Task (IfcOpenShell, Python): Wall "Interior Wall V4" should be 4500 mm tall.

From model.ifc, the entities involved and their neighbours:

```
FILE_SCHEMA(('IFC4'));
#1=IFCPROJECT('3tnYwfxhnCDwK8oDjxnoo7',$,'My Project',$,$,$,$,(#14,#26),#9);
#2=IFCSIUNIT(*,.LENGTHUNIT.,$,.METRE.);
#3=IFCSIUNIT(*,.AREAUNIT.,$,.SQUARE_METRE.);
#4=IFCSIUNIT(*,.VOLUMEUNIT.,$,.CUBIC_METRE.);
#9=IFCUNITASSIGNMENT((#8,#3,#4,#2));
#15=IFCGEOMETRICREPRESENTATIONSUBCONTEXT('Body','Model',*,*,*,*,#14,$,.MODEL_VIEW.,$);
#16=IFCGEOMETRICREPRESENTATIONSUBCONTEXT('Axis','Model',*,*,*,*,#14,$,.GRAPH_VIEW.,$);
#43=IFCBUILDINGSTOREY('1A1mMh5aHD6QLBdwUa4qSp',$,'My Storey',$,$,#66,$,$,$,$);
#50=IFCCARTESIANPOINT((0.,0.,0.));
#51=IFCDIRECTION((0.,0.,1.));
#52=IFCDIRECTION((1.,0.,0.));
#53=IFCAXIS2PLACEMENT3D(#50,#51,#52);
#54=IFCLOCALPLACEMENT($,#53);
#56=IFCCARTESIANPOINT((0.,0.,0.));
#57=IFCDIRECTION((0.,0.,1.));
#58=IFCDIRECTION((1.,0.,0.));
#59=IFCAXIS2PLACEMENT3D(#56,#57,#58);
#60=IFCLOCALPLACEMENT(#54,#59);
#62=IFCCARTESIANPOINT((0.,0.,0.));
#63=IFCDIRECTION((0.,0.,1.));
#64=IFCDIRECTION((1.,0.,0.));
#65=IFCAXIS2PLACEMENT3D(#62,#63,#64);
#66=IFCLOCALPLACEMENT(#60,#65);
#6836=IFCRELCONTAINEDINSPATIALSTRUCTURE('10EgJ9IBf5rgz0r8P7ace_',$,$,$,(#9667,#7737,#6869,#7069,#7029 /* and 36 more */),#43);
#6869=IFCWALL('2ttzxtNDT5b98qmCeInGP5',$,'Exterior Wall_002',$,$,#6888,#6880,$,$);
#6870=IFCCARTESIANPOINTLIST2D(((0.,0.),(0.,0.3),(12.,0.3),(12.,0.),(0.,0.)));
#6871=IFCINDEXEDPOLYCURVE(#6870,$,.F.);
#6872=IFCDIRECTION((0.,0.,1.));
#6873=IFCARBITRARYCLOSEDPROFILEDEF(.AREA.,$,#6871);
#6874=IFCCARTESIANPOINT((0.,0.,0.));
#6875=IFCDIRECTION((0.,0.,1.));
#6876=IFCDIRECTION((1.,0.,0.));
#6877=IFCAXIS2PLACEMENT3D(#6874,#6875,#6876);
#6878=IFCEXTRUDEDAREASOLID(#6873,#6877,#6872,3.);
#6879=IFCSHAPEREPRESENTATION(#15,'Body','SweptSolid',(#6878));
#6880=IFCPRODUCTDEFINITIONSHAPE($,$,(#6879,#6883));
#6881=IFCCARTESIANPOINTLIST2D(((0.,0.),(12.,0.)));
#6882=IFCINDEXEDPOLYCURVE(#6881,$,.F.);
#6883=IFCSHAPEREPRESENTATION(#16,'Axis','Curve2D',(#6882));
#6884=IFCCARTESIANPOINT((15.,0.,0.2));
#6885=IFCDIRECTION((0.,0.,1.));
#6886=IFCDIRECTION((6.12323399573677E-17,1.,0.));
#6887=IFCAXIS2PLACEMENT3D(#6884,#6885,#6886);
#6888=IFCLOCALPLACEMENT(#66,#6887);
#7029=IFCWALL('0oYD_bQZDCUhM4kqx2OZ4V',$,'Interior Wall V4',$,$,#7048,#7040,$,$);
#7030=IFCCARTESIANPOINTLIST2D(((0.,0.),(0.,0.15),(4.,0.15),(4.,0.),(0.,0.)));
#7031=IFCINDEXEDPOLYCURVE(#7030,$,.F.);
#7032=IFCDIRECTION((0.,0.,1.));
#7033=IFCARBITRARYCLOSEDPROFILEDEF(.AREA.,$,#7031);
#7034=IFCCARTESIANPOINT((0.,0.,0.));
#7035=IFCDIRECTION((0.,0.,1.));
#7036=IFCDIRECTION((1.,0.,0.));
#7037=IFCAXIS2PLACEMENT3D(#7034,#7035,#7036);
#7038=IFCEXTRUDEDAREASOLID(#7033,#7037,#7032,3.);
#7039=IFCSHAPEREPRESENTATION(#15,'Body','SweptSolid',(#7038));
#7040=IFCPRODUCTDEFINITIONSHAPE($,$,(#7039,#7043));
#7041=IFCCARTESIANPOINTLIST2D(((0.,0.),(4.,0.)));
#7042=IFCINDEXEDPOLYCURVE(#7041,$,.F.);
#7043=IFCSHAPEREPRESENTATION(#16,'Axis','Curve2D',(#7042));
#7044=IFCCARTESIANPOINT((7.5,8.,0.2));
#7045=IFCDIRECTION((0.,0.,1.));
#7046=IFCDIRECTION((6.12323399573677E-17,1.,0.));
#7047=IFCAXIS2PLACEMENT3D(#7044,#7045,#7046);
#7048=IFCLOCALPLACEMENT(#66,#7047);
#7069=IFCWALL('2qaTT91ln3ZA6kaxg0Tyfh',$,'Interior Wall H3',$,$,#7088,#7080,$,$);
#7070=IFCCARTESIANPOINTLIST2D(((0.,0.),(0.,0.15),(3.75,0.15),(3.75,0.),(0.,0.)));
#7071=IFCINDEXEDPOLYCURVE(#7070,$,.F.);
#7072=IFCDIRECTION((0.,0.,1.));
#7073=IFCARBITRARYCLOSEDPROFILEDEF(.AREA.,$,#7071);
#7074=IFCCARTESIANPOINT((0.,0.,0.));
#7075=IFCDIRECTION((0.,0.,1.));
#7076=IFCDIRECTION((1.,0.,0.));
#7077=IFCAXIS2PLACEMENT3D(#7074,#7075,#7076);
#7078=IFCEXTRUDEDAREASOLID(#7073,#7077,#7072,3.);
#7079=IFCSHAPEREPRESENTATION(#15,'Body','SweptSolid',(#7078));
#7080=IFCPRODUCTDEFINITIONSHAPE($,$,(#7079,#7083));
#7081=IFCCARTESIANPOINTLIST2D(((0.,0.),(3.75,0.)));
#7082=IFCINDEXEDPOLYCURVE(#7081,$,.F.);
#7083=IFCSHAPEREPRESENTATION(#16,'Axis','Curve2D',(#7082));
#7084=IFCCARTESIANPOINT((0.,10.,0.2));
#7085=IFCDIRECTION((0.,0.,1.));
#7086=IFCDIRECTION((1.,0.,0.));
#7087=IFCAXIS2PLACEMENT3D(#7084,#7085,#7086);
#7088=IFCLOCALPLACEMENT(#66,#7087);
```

```python
import ifcopenshell
import ifcopenshell.geom
import ifcopenshell.util.representation
import ifcopenshell.util.shape
import ifcopenshell.util.unit

model = ifcopenshell.open("model.ifc")
unit_scale = ifcopenshell.util.unit.calculate_unit_scale(model)
settings = ifcopenshell.geom.settings()


def volume(element):
    """Net volume in cubic metres, openings subtracted."""
    shape = ifcopenshell.geom.create_shape(settings, element)
    return ifcopenshell.util.shape.get_volume(shape.geometry)


wall = model.by_guid("0oYD_bQZDCUhM4kqx2OZ4V")
before = volume(wall)

body = ifcopenshell.util.representation.get_representation(wall, "Model", "Body")
solid = body.Items[0]
old_height = solid.Depth
solid.Depth = 4.5 / unit_scale
after = volume(wall)

print(f"height {old_height:g} -> {solid.Depth:g}, volume {before:.3f} -> {after:.3f} m3")

model.write("model_edited.ifc")
```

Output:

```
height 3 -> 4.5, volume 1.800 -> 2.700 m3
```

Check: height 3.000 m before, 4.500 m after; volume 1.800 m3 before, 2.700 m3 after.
